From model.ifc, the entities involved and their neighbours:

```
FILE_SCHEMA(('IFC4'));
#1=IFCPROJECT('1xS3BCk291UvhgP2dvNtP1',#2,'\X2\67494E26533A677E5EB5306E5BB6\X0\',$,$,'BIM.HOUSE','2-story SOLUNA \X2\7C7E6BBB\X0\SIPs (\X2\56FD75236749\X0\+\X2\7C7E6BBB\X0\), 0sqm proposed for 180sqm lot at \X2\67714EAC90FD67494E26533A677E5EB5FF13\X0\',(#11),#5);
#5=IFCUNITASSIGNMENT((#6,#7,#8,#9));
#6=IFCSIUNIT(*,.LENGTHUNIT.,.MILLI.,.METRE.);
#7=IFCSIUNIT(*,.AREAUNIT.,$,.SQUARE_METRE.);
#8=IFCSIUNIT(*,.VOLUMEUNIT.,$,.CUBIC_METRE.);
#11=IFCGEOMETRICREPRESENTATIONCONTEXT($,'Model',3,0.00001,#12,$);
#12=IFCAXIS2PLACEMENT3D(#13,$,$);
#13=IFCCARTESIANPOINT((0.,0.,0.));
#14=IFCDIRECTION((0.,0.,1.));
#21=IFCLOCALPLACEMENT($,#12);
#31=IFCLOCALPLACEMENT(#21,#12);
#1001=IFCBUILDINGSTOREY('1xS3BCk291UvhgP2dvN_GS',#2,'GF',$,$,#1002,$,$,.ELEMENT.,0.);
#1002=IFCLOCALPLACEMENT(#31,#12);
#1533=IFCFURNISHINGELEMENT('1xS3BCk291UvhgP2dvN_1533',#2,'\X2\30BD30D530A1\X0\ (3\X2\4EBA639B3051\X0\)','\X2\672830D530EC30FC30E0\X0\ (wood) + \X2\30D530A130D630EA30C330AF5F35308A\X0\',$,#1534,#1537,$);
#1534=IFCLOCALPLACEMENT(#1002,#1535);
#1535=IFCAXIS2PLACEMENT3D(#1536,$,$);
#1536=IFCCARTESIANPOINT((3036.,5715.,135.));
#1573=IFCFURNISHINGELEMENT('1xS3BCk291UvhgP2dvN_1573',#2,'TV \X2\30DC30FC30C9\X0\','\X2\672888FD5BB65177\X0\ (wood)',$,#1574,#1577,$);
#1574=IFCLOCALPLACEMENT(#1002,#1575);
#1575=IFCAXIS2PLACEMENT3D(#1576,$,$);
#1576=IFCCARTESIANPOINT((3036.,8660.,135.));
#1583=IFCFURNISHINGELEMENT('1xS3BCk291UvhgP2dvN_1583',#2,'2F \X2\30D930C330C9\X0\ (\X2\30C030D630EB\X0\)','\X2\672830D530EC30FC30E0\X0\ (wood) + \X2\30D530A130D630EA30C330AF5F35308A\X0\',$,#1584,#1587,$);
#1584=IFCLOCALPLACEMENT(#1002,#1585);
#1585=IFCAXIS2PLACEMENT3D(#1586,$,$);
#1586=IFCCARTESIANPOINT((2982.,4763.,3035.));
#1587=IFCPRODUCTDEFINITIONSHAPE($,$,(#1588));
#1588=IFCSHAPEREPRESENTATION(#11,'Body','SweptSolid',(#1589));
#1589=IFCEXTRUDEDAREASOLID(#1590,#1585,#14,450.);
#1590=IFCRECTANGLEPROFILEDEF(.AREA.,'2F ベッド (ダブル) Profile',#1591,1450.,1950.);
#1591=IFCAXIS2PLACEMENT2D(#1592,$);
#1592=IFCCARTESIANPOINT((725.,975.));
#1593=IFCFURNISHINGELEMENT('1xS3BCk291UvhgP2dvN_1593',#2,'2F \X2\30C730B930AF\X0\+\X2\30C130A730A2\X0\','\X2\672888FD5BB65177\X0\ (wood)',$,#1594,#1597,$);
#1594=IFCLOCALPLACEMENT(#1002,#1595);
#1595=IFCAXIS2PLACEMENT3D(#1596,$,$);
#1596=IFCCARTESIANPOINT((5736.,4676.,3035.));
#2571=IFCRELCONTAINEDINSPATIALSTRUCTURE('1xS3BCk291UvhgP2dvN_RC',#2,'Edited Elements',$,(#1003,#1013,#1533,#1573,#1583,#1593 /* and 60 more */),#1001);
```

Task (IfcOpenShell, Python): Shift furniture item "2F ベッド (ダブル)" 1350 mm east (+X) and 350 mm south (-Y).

```python
import ifcopenshell
import ifcopenshell.api.geometry
import ifcopenshell.util.placement
import ifcopenshell.util.unit

model = ifcopenshell.open("model.ifc")
unit_scale = ifcopenshell.util.unit.calculate_unit_scale(model)

item = model.by_id(1583)
matrix = ifcopenshell.util.placement.get_local_placement(item.ObjectPlacement)
matrix[0, 3] += 1.35 / unit_scale
matrix[1, 3] -= 0.35 / unit_scale
ifcopenshell.api.geometry.edit_object_placement(model, product=item, matrix=matrix, is_si=False)

print(ifcopenshell.util.placement.get_local_placement(item.ObjectPlacement).round(3) + 0.0)

model.write("model_edited.ifc")
```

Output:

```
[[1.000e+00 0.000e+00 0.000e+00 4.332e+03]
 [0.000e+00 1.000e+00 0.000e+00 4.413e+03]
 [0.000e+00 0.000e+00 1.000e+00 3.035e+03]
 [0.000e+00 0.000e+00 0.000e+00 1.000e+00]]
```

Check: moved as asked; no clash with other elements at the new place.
